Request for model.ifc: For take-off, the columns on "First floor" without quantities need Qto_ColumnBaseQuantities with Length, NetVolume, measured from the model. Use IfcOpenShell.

First a look at what the model holds.

```python
import ifcopenshell
import ifcopenshell.util.element
import ifcopenshell.util.unit

model = ifcopenshell.open("model.ifc")
print(model.schema)
for unit_type in ("LENGTHUNIT", "AREAUNIT", "VOLUMEUNIT"):
    print(unit_type, ifcopenshell.util.unit.calculate_unit_scale(model, unit_type))
storey = next(s for s in model.by_type("IfcBuildingStorey") if s.Name == "First floor")
columns = [e for e in ifcopenshell.util.element.get_decomposition(storey) if e.is_a("IfcColumn")]
for e in sorted(columns, key=lambda e: e.id()):
    print(e.id(), e.is_a(), e.Name, list(ifcopenshell.util.element.get_psets(e, qtos_only=True)), sep=" | ")
```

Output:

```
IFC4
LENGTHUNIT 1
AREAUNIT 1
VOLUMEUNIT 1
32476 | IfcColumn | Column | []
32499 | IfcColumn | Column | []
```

```python
import ifcopenshell
import ifcopenshell.api.pset
import ifcopenshell.geom
import ifcopenshell.util.element
import ifcopenshell.util.shape
import ifcopenshell.util.unit

model = ifcopenshell.open("model.ifc")
unit_scale = ifcopenshell.util.unit.calculate_unit_scale(model)
volume_scale = ifcopenshell.util.unit.calculate_unit_scale(model, "VOLUMEUNIT")
settings = ifcopenshell.geom.settings()

storey = next(s for s in model.by_type("IfcBuildingStorey") if s.Name == "First floor")
columns = [e for e in ifcopenshell.util.element.get_decomposition(storey) if e.is_a("IfcColumn")]

for e in sorted(columns, key=lambda e: e.id()):
    if ifcopenshell.util.element.get_psets(e, qtos_only=True, should_inherit=False):
        continue
    # Geometry comes back in metres, in the element's own axes.
    shape = ifcopenshell.geom.create_shape(settings, e)
    values = {
        "Length": ifcopenshell.util.shape.get_z(shape.geometry) / unit_scale,
        "NetVolume": ifcopenshell.util.shape.get_volume(shape.geometry) / volume_scale,
    }
    qto = ifcopenshell.api.pset.add_qto(model, product=e, name="Qto_ColumnBaseQuantities")
    ifcopenshell.api.pset.edit_qto(model, qto=qto, properties=values)
    print(e.id(), {k: round(v, 3) for k, v in values.items()})

model.write("model_rev.ifc")
```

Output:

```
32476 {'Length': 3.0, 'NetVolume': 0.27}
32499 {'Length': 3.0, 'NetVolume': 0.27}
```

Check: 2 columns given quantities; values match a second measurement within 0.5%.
